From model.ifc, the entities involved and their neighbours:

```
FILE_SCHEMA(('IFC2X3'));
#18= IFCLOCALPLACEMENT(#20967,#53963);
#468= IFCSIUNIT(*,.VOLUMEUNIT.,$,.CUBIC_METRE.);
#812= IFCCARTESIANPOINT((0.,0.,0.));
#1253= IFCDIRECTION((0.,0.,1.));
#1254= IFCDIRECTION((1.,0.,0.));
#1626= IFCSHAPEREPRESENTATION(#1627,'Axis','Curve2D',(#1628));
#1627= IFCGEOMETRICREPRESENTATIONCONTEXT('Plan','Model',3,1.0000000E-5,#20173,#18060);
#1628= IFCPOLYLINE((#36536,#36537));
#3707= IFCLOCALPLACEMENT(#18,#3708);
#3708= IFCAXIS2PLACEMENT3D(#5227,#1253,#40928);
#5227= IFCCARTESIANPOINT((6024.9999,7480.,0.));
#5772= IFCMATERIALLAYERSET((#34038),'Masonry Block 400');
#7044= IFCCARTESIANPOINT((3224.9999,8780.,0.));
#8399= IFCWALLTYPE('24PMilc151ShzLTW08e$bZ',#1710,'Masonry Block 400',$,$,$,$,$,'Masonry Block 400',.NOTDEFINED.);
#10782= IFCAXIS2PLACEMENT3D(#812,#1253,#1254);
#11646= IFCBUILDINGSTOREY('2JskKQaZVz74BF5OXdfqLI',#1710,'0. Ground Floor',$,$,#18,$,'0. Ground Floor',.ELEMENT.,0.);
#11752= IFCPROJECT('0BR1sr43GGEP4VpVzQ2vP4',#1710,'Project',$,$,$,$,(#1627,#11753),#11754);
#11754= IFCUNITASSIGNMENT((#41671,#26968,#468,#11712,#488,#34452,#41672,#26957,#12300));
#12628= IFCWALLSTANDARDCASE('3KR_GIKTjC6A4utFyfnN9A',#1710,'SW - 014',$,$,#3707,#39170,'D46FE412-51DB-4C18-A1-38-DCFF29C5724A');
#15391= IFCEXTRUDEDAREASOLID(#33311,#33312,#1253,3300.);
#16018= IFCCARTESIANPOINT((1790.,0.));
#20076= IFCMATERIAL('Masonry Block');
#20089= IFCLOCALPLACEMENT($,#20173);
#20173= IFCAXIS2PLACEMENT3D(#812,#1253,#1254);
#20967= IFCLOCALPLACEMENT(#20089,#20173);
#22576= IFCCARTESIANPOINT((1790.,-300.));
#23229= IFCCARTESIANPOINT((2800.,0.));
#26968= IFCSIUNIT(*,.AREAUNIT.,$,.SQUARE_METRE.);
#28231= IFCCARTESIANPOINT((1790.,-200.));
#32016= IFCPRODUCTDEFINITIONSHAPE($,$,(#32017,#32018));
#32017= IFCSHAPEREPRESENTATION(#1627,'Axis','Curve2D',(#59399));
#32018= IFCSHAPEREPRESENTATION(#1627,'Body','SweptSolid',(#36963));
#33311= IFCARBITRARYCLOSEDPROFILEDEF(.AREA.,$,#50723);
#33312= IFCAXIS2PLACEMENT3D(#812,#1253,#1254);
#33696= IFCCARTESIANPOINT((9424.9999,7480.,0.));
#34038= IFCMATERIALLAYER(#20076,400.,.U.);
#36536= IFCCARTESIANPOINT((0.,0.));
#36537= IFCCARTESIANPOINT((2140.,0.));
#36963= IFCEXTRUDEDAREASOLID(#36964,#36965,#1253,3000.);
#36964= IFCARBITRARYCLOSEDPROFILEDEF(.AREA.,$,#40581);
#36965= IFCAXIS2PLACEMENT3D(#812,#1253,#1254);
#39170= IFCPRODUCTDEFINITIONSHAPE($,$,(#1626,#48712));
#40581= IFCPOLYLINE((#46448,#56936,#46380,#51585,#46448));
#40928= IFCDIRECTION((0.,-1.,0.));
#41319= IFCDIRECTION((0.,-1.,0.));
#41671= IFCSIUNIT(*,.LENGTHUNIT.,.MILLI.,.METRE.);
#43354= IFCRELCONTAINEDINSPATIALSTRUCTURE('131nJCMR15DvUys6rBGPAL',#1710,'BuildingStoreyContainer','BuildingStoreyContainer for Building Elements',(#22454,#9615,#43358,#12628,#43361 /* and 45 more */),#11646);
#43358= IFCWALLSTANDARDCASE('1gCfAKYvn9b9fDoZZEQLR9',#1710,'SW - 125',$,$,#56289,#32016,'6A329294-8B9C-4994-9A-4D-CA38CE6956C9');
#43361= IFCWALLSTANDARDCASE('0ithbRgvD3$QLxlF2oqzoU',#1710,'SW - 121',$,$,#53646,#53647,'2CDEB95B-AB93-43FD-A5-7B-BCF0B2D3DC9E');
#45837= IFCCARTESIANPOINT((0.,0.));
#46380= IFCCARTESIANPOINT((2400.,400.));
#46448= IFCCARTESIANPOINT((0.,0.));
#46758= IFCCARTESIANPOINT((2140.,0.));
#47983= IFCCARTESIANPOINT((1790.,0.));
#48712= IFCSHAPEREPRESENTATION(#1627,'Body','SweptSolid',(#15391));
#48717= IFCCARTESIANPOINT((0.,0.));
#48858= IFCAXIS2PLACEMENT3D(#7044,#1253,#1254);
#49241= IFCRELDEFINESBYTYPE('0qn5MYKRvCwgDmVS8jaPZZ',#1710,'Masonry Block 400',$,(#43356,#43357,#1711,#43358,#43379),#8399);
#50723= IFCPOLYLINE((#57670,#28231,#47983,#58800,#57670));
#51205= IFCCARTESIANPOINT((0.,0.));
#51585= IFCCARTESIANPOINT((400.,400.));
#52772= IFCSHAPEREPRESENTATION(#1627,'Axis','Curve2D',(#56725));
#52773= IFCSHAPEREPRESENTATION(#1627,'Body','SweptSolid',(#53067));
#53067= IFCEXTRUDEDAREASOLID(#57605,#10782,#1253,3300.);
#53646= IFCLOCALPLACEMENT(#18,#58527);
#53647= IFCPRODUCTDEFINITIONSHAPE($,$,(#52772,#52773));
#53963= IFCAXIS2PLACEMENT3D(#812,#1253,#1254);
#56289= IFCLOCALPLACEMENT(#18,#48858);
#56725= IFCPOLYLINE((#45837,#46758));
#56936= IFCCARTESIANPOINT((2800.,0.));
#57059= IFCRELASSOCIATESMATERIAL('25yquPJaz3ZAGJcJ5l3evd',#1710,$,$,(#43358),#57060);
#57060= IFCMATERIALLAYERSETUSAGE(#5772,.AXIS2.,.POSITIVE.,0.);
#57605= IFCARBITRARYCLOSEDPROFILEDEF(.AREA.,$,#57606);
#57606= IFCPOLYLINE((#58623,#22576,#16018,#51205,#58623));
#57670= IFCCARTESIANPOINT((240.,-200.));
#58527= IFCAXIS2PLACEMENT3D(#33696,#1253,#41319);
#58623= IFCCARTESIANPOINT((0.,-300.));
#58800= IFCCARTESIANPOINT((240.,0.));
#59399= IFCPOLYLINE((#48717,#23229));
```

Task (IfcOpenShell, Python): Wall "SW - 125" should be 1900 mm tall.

```python
import ifcopenshell
import ifcopenshell.geom
import ifcopenshell.util.shape
import ifcopenshell.util.unit

model = ifcopenshell.open("model.ifc")
unit_scale = ifcopenshell.util.unit.calculate_unit_scale(model)
settings = ifcopenshell.geom.settings()


def volume(element):
    """Net volume in cubic metres, openings subtracted."""
    shape = ifcopenshell.geom.create_shape(settings, element)
    return ifcopenshell.util.shape.get_volume(shape.geometry)


wall = model.by_id(43358)
before = volume(wall)

body = next(r for r in wall.Representation.Representations if r.RepresentationIdentifier == "Body")
solid = body.Items[0]
old_height = solid.Depth
solid.Depth = 1.9 / unit_scale
after = volume(wall)

print(f"height {old_height:g} -> {solid.Depth:g}, volume {before:.3f} -> {after:.3f} m3")

model.write("model_updated.ifc")
```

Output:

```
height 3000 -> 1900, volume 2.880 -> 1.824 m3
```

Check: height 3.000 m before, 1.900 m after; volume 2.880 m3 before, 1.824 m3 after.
